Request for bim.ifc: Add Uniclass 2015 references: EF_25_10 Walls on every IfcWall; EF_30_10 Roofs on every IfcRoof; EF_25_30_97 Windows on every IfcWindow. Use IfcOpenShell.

First a look at what the model holds.

```python
import ifcopenshell

model = ifcopenshell.open("bim.ifc")
print(model.schema)
print("classifications:", [c.Name for c in model.by_type("IfcClassification")])
for ifc_class in ("IfcDoor", "IfcRoof", "IfcStair", "IfcWall", "IfcWindow"):
    print(ifc_class, len(model.by_type(ifc_class)))
```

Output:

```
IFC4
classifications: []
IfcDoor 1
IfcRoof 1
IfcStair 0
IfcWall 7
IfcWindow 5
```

```python
import ifcopenshell
import ifcopenshell.api.classification

model = ifcopenshell.open("bim.ifc")

system = ifcopenshell.api.classification.add_classification(model, classification="Uniclass 2015")

codes = {
    "IfcWall": ("EF_25_10", "Walls"),
    "IfcRoof": ("EF_30_10", "Roofs"),
    "IfcWindow": ("EF_25_30_97", "Windows"),
}
for ifc_class, (code, name) in codes.items():
    products = model.by_type(ifc_class)
    ifcopenshell.api.classification.add_reference(
        model, products=products, classification=system, identification=code, name=name
    )
    print(code, len(products))

model.write("bim-out.ifc")
```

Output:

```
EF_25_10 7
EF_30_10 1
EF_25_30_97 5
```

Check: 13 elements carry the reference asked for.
